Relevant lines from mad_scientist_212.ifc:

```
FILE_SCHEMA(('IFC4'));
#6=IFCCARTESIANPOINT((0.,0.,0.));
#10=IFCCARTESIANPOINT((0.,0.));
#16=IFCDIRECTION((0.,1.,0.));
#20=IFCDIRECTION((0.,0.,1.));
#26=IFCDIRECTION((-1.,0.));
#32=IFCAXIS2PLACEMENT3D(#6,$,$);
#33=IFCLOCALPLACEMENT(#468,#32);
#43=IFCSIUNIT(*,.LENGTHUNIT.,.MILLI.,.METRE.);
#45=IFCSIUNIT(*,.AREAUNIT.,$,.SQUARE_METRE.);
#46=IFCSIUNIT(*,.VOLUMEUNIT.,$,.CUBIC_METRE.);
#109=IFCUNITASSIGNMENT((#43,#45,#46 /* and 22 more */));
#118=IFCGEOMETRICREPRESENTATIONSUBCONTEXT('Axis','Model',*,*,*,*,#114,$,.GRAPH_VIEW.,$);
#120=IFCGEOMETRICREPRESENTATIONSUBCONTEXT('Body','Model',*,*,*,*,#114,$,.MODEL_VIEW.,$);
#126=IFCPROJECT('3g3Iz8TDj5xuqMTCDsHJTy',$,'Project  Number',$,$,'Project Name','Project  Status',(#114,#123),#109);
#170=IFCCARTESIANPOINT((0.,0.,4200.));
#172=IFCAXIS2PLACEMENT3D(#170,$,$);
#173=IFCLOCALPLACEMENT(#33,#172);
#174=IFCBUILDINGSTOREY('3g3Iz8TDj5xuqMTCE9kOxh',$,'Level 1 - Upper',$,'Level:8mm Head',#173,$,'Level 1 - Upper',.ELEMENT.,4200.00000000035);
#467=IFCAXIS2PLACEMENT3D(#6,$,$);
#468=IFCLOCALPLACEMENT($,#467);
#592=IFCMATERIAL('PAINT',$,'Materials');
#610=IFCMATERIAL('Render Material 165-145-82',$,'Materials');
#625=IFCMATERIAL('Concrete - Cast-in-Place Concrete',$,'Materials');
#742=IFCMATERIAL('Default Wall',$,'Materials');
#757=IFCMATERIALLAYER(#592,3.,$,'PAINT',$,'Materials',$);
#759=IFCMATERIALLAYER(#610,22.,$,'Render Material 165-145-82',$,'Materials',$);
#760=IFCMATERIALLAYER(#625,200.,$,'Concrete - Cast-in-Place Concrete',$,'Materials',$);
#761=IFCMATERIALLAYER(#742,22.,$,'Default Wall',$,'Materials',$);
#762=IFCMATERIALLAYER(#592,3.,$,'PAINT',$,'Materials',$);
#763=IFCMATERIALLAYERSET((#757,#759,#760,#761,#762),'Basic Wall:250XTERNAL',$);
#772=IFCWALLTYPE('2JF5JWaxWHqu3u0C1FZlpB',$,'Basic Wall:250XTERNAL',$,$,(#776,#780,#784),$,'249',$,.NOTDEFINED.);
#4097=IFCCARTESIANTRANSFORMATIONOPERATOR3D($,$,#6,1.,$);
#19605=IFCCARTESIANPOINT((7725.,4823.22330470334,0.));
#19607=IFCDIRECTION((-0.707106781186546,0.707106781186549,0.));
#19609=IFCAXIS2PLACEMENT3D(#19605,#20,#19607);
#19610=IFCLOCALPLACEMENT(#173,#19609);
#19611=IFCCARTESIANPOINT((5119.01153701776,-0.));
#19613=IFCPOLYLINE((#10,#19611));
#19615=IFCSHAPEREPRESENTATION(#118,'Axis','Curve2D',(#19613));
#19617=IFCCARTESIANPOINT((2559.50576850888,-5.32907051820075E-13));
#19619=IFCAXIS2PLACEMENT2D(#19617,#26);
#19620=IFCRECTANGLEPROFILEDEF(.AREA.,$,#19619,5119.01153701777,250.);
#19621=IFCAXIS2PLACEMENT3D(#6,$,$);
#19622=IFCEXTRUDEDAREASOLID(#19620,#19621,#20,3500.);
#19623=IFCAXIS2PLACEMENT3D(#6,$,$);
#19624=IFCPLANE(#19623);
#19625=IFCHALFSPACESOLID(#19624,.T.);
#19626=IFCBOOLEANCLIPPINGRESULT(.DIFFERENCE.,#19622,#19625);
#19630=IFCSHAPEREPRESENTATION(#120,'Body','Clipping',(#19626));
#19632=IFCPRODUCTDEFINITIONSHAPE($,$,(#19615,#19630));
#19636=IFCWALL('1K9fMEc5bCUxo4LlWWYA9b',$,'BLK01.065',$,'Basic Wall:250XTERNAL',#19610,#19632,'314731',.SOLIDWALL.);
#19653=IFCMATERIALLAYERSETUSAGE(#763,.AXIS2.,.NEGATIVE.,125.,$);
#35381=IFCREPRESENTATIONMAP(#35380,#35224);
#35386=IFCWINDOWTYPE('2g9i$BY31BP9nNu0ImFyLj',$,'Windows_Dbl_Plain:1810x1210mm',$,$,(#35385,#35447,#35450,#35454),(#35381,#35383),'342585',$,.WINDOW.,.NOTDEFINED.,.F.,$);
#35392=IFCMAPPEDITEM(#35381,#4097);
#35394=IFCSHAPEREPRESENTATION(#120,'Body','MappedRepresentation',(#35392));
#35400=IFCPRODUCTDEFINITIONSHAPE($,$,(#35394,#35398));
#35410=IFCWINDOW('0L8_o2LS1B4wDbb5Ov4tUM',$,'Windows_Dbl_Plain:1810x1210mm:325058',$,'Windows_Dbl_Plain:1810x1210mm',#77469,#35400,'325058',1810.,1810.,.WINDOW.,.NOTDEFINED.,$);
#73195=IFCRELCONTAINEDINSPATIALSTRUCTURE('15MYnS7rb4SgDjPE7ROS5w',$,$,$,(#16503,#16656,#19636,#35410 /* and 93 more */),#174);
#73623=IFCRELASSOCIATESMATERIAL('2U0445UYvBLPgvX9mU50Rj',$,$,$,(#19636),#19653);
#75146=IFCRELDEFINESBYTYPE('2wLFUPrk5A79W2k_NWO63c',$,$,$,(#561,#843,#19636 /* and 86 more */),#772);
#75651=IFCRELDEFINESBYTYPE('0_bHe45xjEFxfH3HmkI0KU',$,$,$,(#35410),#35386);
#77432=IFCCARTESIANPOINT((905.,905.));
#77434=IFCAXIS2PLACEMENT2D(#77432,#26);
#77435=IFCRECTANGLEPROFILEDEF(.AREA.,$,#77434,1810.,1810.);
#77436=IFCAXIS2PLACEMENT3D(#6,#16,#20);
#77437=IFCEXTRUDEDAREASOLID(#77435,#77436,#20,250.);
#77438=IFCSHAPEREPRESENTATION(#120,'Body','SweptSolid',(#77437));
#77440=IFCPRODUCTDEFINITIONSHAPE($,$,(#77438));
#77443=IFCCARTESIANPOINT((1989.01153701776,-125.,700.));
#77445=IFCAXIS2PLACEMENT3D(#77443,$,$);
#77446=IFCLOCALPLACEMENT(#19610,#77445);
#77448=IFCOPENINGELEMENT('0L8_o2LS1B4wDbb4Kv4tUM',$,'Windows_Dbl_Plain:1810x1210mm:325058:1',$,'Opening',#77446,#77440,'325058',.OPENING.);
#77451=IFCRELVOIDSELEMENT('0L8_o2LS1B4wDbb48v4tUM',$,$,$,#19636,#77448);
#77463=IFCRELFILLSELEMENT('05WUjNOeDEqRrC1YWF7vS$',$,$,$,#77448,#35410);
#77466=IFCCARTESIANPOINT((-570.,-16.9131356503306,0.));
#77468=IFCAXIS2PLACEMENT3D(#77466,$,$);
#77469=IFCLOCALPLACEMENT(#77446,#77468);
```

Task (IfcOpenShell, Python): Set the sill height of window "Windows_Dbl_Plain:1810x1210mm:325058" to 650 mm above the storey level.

```python
import numpy as np
import ifcopenshell
import ifcopenshell.api.geometry
import ifcopenshell.geom
import ifcopenshell.util.element
import ifcopenshell.util.placement
import ifcopenshell.util.shape
import ifcopenshell.util.unit

model = ifcopenshell.open("mad_scientist_212.ifc")
unit_scale = ifcopenshell.util.unit.calculate_unit_scale(model)

window = model.by_guid("0L8_o2LS1B4wDbb5Ov4tUM")
opening = window.FillsVoids[0].RelatingOpeningElement
storey = ifcopenshell.util.element.get_container(window, ifc_class="IfcBuildingStorey")
level = ifcopenshell.util.placement.get_local_placement(storey.ObjectPlacement)[2, 3]

# The opening's origin need not be at the sill, so measure its lowest point.
shape = ifcopenshell.geom.create_shape(ifcopenshell.geom.settings(), opening)
bottom = ifcopenshell.util.shape.get_shape_bottom_elevation(shape, shape.geometry) / unit_scale
dz = level + 0.65 / unit_scale - bottom

shift = np.array([0.0, 0.0, dz])
# The window is placed relative to its opening, so it follows when the opening moves.
matrix = ifcopenshell.util.placement.get_local_placement(opening.ObjectPlacement)
matrix[:3, 3] += shift
ifcopenshell.api.geometry.edit_object_placement(
    model, product=opening, matrix=matrix, is_si=False, should_transform_children=True
)

print(f"moved by {dz * unit_scale:+.3f} m")

model.write("mad_scientist_212-out.ifc")
```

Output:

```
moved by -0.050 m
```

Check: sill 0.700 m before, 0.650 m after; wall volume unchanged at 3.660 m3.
